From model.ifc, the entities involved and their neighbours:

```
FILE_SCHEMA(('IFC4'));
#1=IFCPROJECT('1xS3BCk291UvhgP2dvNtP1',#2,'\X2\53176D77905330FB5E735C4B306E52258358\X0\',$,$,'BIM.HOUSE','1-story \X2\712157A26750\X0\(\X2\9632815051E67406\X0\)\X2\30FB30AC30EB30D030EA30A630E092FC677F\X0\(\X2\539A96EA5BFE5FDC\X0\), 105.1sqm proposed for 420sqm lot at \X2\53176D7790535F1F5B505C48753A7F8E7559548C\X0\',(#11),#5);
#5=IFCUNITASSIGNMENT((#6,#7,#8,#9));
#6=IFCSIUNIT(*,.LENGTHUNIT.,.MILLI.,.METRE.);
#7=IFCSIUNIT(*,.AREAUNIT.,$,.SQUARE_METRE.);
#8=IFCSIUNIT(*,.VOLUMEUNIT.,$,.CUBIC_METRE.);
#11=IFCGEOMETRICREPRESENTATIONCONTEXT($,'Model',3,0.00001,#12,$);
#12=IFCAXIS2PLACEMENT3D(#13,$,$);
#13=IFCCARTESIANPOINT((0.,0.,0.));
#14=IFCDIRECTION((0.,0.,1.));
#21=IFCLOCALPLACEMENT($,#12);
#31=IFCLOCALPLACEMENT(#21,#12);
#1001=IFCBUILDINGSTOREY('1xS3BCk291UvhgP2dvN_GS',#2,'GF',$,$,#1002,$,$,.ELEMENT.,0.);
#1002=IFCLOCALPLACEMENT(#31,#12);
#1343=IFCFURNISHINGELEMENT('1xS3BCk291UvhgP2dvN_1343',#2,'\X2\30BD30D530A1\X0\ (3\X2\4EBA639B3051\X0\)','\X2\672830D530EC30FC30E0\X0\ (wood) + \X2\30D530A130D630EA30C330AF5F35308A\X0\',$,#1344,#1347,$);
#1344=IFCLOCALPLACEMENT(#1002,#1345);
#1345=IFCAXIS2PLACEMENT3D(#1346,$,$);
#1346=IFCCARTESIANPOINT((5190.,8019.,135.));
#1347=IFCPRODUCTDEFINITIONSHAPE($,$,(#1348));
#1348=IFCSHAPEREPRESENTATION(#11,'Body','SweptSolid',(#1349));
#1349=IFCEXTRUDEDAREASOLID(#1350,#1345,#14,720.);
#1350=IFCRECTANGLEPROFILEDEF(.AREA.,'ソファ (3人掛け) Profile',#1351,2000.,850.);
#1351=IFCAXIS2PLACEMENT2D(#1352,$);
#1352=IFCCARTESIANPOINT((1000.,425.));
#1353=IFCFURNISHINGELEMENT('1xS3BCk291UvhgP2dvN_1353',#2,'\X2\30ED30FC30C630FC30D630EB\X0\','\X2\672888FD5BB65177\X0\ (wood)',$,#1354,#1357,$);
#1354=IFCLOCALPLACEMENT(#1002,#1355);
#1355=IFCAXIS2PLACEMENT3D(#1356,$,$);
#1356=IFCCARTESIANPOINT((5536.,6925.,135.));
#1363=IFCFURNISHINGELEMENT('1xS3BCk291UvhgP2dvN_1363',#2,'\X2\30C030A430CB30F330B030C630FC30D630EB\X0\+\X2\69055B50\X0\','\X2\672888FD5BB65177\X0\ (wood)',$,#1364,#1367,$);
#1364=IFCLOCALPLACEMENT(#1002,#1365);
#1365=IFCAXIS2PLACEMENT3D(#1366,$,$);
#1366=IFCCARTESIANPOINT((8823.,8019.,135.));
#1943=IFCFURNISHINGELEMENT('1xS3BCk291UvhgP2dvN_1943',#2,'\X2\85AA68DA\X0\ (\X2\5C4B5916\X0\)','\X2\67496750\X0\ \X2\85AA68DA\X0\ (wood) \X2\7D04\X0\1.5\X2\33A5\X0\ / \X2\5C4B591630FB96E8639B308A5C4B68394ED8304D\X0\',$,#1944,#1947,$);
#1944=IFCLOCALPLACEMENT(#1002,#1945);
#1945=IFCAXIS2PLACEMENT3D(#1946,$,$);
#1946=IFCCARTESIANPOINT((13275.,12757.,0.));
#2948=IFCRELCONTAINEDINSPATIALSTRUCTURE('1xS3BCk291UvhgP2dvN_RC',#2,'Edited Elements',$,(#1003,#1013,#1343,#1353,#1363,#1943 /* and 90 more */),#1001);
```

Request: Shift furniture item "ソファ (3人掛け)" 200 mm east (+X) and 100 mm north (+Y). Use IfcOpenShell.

```python
import ifcopenshell
import ifcopenshell.api.geometry
import ifcopenshell.util.placement

model = ifcopenshell.open("model.ifc")

item = model.by_guid("1xS3BCk291UvhgP2dvN_1343")
matrix = ifcopenshell.util.placement.get_local_placement(item.ObjectPlacement)
matrix[0, 3] += 200.0
matrix[1, 3] += 100.0
ifcopenshell.api.geometry.edit_object_placement(model, product=item, matrix=matrix, is_si=False)

print(ifcopenshell.util.placement.get_local_placement(item.ObjectPlacement).round(3) + 0.0)

model.write("model_v2.ifc")
```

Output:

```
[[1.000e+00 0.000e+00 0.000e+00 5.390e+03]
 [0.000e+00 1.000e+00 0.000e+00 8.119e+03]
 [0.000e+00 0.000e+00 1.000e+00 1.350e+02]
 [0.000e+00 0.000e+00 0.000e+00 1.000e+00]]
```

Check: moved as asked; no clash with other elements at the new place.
